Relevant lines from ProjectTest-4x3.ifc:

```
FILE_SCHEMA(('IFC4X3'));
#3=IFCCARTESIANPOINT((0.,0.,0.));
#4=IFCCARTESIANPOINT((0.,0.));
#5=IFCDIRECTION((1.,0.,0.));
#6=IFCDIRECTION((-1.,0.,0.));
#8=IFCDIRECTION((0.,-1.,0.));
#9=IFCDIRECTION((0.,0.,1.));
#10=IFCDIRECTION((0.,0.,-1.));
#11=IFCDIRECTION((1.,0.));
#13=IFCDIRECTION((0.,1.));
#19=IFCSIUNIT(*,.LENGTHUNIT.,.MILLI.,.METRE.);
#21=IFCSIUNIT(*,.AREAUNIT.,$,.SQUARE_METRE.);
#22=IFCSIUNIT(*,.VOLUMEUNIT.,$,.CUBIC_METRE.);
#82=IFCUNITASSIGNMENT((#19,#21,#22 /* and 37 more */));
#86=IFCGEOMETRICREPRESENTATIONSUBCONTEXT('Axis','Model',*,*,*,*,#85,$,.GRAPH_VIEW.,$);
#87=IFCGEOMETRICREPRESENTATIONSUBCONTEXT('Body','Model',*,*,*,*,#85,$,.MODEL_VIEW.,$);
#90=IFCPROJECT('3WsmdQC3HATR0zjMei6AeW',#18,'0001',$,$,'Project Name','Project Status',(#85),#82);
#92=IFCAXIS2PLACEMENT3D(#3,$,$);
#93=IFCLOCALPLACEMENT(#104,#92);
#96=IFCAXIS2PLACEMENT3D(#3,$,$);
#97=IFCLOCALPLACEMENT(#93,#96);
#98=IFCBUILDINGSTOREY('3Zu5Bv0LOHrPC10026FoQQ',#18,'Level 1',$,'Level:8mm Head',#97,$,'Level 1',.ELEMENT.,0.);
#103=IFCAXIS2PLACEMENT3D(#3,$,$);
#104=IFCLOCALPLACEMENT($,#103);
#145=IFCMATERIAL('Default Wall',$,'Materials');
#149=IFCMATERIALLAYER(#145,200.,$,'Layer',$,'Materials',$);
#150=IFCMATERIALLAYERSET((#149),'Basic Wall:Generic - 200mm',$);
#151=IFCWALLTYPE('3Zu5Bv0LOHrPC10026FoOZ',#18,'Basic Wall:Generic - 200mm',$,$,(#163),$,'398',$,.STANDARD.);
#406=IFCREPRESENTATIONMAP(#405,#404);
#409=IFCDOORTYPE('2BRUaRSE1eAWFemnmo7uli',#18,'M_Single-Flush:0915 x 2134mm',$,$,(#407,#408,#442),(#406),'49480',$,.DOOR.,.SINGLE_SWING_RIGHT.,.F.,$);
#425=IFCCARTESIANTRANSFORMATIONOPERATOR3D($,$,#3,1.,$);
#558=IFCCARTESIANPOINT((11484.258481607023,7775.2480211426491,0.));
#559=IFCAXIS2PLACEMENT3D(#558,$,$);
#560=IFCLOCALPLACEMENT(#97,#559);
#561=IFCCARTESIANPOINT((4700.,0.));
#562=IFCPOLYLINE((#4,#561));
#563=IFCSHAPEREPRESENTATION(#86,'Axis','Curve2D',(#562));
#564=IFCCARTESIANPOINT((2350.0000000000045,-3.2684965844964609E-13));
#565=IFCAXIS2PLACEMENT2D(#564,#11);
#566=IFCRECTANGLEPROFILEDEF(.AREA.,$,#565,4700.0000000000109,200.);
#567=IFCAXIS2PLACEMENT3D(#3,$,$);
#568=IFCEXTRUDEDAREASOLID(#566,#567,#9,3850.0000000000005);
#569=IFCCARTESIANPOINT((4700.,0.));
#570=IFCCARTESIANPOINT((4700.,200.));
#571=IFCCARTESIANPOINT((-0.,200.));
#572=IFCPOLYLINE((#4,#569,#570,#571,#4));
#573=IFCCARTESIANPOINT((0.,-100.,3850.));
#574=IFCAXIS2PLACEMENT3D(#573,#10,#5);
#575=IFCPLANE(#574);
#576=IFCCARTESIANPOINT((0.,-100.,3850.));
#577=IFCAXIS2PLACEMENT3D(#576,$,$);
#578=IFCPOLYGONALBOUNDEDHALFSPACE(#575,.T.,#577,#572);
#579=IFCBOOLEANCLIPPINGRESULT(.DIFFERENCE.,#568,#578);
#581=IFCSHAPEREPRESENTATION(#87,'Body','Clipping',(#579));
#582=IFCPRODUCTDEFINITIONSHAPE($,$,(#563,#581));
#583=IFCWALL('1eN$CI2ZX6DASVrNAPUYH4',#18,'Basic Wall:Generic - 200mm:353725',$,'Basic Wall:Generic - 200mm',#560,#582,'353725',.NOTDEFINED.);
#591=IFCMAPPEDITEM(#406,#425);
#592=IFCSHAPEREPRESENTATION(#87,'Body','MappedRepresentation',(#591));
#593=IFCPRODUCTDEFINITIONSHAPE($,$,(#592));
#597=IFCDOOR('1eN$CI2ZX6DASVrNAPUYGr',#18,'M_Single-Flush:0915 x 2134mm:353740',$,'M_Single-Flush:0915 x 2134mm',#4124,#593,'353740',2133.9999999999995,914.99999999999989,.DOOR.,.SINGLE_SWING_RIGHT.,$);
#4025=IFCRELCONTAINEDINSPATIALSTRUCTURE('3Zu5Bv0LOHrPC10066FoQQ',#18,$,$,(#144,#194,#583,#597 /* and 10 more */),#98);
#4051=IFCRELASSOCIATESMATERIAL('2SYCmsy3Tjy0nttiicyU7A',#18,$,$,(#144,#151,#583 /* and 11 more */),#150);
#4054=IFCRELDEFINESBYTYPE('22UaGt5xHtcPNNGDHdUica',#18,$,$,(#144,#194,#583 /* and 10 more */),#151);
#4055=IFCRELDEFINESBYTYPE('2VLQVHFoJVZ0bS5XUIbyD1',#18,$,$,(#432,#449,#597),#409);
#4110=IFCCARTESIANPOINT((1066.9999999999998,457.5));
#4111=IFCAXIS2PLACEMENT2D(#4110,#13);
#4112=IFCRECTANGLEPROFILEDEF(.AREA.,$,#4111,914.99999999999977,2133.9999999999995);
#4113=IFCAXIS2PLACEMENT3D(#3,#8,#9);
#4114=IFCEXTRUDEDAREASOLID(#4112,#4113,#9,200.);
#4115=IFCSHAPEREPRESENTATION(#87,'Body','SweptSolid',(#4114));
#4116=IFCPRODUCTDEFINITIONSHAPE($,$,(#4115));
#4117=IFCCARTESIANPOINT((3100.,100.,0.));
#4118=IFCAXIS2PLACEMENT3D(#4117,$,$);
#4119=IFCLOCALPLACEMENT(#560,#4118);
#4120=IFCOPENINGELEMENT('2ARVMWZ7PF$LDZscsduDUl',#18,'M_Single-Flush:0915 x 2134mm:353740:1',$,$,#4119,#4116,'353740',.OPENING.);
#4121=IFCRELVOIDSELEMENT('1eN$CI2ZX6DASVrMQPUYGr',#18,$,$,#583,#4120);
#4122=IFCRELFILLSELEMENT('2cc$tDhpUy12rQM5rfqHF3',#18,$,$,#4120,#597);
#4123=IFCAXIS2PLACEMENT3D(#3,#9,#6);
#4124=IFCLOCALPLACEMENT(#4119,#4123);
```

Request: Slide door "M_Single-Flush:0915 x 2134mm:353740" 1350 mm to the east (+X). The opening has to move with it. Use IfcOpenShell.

```python
import ifcopenshell
import ifcopenshell.api.geometry
import ifcopenshell.util.placement

model = ifcopenshell.open("ProjectTest-4x3.ifc")

door = model.by_guid("1eN$CI2ZX6DASVrNAPUYGr")
opening = door.FillsVoids[0].RelatingOpeningElement
wall = opening.VoidsElements[0].RelatingBuildingElement

wall_matrix = ifcopenshell.util.placement.get_local_placement(wall.ObjectPlacement)
shift = wall_matrix[:3, 0] * 1350.0
before = ifcopenshell.util.placement.get_local_placement(door.ObjectPlacement)[:3, 3].copy()

# The door is placed relative to its opening, so it follows when the opening moves.
matrix = ifcopenshell.util.placement.get_local_placement(opening.ObjectPlacement)
matrix[:3, 3] += shift
ifcopenshell.api.geometry.edit_object_placement(
    model, product=opening, matrix=matrix, is_si=False, should_transform_children=True
)

after = ifcopenshell.util.placement.get_local_placement(door.ObjectPlacement)[:3, 3]
print("door moved by", (after - before).round(3) + 0.0)

model.write("ProjectTest-4x3_v2.ifc")
```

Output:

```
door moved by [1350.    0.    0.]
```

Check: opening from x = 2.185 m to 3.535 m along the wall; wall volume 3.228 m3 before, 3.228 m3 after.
